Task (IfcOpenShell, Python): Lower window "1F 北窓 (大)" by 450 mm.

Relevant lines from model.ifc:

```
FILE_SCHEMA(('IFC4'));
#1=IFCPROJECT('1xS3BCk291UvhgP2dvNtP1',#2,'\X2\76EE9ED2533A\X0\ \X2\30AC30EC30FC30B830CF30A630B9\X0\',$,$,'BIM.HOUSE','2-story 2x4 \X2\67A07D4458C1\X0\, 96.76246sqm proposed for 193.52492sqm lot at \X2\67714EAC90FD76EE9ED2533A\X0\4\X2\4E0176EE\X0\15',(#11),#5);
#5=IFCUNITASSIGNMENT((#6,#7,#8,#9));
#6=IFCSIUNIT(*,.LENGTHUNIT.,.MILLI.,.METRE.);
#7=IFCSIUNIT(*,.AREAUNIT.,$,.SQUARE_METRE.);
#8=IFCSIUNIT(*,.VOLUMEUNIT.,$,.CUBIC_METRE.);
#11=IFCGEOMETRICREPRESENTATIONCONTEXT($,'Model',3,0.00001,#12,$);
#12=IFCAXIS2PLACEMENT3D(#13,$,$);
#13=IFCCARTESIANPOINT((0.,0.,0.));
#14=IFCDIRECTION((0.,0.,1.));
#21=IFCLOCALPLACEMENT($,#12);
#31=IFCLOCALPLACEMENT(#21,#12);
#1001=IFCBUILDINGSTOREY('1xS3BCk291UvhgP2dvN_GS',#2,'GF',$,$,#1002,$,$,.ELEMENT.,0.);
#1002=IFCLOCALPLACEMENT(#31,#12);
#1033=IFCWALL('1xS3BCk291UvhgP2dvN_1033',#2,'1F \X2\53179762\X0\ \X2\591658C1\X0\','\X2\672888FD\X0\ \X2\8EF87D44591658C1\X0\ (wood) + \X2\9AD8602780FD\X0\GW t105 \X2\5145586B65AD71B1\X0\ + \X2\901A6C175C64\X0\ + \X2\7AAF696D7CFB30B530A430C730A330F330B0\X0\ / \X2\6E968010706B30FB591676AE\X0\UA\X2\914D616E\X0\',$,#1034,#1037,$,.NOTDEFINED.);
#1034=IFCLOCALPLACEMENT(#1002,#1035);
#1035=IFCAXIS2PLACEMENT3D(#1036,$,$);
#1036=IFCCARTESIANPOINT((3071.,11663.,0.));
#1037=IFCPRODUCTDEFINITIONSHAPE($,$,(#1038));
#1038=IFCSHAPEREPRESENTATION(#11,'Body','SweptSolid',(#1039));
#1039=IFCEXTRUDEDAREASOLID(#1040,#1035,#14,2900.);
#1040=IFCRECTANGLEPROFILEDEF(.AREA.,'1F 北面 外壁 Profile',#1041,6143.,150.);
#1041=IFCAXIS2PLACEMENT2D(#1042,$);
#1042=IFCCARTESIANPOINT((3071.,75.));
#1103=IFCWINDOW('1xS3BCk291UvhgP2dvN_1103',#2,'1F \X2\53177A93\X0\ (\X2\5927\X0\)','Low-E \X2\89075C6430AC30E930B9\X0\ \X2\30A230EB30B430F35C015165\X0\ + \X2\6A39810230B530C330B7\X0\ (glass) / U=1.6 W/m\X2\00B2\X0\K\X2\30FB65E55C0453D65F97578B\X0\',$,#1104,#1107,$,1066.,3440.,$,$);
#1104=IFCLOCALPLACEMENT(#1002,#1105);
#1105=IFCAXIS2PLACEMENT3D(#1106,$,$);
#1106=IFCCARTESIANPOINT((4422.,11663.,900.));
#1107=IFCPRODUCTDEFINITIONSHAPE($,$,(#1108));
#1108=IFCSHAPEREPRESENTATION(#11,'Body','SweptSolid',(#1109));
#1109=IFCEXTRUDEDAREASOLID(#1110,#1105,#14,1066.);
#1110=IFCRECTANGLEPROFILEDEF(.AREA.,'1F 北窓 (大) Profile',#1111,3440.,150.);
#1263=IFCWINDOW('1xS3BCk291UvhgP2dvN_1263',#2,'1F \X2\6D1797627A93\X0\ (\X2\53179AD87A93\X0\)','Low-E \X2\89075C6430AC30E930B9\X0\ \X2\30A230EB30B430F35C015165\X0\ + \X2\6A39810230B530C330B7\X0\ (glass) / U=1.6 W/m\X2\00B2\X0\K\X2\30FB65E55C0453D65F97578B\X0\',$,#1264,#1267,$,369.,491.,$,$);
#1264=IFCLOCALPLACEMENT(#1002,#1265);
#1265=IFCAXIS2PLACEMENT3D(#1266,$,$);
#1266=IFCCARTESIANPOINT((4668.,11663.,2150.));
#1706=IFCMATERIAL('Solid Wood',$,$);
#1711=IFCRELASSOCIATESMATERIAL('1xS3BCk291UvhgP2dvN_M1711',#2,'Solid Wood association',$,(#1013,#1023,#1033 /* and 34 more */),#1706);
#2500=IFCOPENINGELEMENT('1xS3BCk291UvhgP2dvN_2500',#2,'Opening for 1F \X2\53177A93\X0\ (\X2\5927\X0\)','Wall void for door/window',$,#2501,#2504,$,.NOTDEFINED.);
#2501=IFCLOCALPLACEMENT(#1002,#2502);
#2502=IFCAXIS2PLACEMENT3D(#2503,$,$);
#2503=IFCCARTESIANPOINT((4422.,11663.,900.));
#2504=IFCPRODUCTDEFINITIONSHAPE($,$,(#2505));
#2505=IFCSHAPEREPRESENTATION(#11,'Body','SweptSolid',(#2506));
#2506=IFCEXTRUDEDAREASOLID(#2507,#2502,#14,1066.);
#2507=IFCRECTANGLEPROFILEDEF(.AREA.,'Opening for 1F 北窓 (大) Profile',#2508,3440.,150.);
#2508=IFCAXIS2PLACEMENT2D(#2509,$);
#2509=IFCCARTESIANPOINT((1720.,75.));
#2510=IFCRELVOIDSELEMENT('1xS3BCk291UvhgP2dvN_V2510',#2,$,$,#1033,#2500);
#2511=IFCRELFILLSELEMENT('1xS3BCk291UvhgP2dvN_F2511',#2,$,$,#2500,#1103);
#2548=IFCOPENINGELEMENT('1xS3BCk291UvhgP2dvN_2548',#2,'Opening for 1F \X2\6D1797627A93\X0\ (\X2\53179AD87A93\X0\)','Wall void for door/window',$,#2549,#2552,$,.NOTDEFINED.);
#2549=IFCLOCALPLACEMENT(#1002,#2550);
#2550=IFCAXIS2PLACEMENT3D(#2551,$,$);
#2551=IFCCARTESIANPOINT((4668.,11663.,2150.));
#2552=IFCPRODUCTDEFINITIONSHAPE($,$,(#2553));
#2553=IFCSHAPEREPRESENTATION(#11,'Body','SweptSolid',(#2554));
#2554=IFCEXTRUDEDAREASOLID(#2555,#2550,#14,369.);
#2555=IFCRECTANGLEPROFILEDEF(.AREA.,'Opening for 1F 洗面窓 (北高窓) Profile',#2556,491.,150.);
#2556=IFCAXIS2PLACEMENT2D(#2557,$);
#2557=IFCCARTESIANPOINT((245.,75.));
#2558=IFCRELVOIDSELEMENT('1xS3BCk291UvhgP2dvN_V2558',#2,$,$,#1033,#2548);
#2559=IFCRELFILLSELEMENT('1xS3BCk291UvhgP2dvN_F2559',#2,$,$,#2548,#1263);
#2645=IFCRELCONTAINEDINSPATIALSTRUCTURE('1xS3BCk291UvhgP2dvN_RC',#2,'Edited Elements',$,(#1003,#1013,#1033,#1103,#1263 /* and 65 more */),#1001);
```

```python
import numpy as np
import ifcopenshell
import ifcopenshell.api.geometry
import ifcopenshell.util.placement
import ifcopenshell.util.unit

model = ifcopenshell.open("model.ifc")
unit_scale = ifcopenshell.util.unit.calculate_unit_scale(model)

window = model.by_guid("1xS3BCk291UvhgP2dvN_1103")
opening = window.FillsVoids[0].RelatingOpeningElement
dz = -0.45 / unit_scale

shift = np.array([0.0, 0.0, dz])
# The window is not placed relative to its opening, so move both.
for product in (opening, window):
    matrix = ifcopenshell.util.placement.get_local_placement(product.ObjectPlacement)
    matrix[:3, 3] += shift
    ifcopenshell.api.geometry.edit_object_placement(model, product=product, matrix=matrix, is_si=False)

print(f"moved by {dz * unit_scale:+.3f} m")

model.write("model_edited.ifc")
```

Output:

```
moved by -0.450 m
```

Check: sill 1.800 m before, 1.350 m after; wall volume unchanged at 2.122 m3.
